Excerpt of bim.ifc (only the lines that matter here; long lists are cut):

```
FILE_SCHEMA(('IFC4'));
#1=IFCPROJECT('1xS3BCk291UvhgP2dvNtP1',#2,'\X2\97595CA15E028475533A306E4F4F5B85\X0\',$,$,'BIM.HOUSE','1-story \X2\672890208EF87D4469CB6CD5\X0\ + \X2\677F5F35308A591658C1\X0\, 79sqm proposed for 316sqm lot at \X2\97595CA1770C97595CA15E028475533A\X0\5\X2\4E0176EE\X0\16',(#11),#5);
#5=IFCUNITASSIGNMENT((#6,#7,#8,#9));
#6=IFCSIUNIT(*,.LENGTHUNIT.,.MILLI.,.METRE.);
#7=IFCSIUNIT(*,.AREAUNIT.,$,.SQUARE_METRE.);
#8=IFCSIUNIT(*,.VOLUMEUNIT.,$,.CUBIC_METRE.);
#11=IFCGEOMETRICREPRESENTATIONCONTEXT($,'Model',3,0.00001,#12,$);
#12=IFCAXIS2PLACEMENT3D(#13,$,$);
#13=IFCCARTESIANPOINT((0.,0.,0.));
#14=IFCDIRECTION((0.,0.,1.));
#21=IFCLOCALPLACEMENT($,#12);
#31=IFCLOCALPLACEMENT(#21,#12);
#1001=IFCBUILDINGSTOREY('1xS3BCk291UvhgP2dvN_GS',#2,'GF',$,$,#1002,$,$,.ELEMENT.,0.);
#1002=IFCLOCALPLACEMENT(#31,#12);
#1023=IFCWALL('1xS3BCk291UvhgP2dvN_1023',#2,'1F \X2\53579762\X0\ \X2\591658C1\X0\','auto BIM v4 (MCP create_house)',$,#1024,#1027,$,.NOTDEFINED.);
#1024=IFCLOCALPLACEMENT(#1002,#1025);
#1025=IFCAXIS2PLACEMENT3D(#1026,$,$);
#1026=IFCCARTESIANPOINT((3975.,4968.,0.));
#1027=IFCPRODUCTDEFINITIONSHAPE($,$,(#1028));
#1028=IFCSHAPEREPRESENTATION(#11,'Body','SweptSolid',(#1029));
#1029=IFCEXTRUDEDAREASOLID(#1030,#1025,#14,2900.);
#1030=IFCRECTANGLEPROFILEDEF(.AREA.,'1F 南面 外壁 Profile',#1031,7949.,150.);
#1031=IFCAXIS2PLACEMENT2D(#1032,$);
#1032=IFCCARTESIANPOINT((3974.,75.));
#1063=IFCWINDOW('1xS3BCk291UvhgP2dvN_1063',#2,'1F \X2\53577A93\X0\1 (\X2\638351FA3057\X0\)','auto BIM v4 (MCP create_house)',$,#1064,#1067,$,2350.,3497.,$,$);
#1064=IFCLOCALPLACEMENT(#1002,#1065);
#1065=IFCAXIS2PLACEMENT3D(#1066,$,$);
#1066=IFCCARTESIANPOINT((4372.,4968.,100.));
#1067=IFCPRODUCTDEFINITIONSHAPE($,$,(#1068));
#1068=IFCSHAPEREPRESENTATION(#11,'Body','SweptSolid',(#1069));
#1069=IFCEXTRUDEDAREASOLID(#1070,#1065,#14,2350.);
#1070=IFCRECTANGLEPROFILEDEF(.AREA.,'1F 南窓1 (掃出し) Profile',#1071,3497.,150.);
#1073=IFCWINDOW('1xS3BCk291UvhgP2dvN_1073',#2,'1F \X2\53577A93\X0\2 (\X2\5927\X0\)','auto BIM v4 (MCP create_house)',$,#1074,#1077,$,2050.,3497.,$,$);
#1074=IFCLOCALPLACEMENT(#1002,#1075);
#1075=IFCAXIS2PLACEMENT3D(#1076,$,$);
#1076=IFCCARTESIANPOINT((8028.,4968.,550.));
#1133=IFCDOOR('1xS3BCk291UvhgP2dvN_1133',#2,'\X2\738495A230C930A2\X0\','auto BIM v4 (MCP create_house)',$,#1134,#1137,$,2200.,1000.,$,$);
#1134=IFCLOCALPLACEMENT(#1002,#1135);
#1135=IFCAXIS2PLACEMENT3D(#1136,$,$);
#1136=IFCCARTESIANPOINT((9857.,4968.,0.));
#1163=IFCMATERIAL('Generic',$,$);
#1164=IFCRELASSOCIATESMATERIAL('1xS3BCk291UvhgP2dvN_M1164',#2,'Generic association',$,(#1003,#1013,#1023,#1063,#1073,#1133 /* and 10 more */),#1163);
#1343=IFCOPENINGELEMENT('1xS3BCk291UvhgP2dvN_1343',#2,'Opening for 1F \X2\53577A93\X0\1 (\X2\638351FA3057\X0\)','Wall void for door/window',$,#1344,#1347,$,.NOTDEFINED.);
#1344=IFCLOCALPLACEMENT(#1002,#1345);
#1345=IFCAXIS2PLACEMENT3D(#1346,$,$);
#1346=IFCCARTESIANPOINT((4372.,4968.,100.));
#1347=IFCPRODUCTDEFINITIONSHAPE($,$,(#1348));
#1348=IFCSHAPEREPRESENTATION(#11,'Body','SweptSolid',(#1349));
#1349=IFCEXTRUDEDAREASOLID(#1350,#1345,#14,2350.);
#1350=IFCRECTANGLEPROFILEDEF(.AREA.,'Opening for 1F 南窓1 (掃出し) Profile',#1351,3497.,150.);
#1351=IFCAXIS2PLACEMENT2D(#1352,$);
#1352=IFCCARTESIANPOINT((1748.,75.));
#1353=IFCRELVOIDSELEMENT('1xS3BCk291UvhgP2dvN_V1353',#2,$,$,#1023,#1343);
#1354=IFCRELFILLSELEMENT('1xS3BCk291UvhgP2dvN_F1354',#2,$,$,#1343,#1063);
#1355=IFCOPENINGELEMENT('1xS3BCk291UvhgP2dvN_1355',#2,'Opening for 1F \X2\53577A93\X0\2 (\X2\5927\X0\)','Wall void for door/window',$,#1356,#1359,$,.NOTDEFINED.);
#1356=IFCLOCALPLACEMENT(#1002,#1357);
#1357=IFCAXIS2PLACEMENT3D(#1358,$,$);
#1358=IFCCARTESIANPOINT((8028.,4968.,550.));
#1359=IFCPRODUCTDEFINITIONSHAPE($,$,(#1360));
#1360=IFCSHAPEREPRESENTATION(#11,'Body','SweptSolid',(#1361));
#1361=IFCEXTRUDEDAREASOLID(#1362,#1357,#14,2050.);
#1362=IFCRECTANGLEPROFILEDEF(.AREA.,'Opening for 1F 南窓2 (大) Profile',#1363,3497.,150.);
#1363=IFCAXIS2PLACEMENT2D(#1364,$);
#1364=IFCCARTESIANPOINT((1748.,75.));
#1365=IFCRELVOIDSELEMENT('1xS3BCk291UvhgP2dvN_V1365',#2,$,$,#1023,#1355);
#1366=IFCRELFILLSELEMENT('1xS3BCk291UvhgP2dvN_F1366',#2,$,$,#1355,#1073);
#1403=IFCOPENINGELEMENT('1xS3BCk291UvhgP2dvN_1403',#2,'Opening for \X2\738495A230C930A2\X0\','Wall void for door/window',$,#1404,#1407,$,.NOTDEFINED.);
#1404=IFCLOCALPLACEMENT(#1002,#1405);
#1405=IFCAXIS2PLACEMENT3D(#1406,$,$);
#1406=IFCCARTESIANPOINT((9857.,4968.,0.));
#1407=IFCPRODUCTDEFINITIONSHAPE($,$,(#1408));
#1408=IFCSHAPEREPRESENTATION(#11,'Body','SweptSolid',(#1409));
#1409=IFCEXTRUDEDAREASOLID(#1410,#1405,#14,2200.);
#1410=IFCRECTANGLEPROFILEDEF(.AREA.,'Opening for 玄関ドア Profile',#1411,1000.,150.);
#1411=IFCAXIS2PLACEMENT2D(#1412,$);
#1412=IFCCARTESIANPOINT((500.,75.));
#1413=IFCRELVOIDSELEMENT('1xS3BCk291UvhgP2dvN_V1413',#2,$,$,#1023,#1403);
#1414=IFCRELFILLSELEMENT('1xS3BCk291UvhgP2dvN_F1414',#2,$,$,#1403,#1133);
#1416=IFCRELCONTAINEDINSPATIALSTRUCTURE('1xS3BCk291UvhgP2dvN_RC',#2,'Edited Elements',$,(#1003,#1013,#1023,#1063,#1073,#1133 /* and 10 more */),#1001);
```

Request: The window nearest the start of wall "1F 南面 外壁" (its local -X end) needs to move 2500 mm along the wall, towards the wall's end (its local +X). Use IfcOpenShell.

```python
import ifcopenshell
import ifcopenshell.api.geometry
import ifcopenshell.util.placement
import ifcopenshell.util.unit

model = ifcopenshell.open("bim.ifc")
unit_scale = ifcopenshell.util.unit.calculate_unit_scale(model)

window = model.by_id(1063)
opening = window.FillsVoids[0].RelatingOpeningElement
wall = opening.VoidsElements[0].RelatingBuildingElement

wall_matrix = ifcopenshell.util.placement.get_local_placement(wall.ObjectPlacement)
shift = wall_matrix[:3, 0] * 2.5 / unit_scale
before = ifcopenshell.util.placement.get_local_placement(window.ObjectPlacement)[:3, 3].copy()

# The window is not placed relative to its opening, so move both.
for product in (opening, window):
    matrix = ifcopenshell.util.placement.get_local_placement(product.ObjectPlacement)
    matrix[:3, 3] += shift
    ifcopenshell.api.geometry.edit_object_placement(model, product=product, matrix=matrix, is_si=False)

after = ifcopenshell.util.placement.get_local_placement(window.ObjectPlacement)[:3, 3]
print("window moved by", (after - before).round(3) + 0.0)

model.write("bim_rev.ifc")
```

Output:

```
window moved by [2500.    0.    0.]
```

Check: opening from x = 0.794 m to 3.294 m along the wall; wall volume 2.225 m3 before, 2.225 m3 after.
